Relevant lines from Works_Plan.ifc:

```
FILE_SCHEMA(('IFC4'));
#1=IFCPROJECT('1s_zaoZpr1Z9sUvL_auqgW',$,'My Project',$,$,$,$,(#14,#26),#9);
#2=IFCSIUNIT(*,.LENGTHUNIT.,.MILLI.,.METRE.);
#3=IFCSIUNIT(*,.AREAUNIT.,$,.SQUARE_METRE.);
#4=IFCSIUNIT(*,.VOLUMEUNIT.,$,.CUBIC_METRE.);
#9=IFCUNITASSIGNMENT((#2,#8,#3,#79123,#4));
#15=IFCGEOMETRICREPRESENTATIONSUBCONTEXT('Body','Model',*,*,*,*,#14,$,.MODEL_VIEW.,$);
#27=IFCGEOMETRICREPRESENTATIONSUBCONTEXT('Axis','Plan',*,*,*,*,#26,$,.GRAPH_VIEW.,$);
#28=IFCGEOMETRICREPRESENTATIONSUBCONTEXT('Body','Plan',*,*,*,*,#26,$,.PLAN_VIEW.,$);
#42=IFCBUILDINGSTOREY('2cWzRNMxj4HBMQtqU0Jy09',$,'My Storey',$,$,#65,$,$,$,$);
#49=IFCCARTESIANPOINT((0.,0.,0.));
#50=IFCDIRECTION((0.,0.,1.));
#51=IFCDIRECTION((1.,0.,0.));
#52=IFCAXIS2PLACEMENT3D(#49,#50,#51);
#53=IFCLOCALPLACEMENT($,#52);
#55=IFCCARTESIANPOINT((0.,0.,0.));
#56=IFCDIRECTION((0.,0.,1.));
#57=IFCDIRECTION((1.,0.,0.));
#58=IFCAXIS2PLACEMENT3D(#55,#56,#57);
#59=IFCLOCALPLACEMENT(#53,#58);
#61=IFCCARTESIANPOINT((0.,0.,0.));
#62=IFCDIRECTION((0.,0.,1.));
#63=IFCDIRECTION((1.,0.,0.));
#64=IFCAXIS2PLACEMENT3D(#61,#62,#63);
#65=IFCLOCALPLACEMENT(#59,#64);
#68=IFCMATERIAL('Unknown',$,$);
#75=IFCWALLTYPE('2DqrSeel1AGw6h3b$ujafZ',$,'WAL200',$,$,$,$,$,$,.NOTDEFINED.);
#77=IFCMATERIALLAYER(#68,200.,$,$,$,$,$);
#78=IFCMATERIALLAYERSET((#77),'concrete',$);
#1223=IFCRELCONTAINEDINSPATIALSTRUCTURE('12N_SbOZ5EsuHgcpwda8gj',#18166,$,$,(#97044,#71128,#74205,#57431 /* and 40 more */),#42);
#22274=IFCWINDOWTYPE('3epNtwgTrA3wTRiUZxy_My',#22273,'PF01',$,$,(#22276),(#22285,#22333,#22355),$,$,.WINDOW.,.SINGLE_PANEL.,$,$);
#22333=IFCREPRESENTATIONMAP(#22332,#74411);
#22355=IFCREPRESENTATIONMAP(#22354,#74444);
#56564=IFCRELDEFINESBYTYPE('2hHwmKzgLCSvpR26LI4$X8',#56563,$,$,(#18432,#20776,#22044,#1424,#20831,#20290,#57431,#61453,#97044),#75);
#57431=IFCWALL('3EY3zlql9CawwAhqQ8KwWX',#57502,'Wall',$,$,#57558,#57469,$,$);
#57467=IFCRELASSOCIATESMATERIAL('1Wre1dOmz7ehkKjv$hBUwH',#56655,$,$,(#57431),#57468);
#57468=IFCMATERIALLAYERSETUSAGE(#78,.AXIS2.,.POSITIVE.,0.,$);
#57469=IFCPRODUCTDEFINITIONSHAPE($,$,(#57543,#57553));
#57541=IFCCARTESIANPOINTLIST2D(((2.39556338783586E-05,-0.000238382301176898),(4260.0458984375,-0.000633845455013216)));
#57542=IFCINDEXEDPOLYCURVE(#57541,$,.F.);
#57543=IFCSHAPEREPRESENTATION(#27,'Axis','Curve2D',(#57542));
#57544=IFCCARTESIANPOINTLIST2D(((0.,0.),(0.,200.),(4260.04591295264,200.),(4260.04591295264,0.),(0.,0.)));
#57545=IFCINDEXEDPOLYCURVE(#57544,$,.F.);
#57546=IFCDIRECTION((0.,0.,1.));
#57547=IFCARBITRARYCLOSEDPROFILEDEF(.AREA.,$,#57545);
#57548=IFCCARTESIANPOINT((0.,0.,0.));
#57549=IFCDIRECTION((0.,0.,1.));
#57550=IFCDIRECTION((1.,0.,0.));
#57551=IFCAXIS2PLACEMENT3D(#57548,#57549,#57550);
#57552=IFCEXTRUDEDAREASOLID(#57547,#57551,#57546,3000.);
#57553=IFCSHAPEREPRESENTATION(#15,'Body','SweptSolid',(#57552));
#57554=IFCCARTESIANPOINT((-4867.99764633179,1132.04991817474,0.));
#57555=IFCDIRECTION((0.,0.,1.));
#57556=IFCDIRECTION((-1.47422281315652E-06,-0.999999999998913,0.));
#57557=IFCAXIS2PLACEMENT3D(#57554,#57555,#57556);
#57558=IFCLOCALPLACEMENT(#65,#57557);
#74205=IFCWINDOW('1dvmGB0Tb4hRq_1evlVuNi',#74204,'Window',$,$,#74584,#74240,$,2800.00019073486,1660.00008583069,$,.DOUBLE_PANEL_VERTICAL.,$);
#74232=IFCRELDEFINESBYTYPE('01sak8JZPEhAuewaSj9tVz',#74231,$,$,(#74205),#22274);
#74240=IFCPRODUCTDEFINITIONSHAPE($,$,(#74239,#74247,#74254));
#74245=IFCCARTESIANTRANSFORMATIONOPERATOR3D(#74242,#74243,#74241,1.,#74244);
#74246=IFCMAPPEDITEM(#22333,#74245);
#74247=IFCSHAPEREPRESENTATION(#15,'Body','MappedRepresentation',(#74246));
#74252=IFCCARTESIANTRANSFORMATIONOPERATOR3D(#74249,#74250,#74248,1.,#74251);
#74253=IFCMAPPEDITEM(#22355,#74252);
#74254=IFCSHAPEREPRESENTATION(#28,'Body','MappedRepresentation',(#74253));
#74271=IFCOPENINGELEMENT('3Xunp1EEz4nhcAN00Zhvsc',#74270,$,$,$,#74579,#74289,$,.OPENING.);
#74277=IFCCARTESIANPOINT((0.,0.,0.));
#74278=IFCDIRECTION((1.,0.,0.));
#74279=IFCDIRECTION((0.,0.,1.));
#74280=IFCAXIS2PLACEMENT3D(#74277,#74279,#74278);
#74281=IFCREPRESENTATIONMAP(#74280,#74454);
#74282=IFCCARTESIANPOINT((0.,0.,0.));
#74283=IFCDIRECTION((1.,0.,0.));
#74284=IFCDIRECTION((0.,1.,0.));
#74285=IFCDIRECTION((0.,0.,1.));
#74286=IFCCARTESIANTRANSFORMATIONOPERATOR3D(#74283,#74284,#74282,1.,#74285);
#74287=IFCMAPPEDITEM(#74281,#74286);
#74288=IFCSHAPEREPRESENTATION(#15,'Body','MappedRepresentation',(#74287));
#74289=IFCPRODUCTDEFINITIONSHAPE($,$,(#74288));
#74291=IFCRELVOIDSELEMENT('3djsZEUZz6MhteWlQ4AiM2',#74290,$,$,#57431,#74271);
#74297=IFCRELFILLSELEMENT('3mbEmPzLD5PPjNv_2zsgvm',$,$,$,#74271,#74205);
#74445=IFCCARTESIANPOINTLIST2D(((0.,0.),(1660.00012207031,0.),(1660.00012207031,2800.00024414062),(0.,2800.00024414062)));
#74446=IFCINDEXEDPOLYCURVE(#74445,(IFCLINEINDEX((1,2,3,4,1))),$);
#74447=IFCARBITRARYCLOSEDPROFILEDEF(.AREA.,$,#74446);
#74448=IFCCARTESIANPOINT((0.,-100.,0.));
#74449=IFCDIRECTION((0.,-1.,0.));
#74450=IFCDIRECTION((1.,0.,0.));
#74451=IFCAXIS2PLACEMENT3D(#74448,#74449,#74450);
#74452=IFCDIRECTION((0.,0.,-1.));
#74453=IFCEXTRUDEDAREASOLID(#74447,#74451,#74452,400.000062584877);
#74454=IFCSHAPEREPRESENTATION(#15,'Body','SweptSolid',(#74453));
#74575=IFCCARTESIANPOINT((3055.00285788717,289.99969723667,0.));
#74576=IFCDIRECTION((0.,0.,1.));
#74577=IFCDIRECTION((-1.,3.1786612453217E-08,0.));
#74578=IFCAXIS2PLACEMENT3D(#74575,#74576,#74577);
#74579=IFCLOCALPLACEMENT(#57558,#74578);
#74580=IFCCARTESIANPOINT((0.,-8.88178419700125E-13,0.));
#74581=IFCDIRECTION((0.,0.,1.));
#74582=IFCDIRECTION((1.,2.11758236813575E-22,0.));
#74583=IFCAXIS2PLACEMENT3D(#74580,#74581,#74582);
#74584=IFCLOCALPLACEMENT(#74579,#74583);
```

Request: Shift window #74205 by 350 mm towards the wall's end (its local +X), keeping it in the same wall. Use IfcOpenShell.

```python
import ifcopenshell
import ifcopenshell.api.geometry
import ifcopenshell.util.placement

model = ifcopenshell.open("Works_Plan.ifc")

window = model.by_id(74205)
opening = window.FillsVoids[0].RelatingOpeningElement
wall = opening.VoidsElements[0].RelatingBuildingElement

wall_matrix = ifcopenshell.util.placement.get_local_placement(wall.ObjectPlacement)
shift = wall_matrix[:3, 0] * 350.0
before = ifcopenshell.util.placement.get_local_placement(window.ObjectPlacement)[:3, 3].copy()

# The window is placed relative to its opening, so it follows when the opening moves.
matrix = ifcopenshell.util.placement.get_local_placement(opening.ObjectPlacement)
matrix[:3, 3] += shift
ifcopenshell.api.geometry.edit_object_placement(
    model, product=opening, matrix=matrix, is_si=False, should_transform_children=True
)

after = ifcopenshell.util.placement.get_local_placement(window.ObjectPlacement)[:3, 3]
print("window moved by", (after - before).round(3) + 0.0)

model.write("Works_Plan-out.ifc")
```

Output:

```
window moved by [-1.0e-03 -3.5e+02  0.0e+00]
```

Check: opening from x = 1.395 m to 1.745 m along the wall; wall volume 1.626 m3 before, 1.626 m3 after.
